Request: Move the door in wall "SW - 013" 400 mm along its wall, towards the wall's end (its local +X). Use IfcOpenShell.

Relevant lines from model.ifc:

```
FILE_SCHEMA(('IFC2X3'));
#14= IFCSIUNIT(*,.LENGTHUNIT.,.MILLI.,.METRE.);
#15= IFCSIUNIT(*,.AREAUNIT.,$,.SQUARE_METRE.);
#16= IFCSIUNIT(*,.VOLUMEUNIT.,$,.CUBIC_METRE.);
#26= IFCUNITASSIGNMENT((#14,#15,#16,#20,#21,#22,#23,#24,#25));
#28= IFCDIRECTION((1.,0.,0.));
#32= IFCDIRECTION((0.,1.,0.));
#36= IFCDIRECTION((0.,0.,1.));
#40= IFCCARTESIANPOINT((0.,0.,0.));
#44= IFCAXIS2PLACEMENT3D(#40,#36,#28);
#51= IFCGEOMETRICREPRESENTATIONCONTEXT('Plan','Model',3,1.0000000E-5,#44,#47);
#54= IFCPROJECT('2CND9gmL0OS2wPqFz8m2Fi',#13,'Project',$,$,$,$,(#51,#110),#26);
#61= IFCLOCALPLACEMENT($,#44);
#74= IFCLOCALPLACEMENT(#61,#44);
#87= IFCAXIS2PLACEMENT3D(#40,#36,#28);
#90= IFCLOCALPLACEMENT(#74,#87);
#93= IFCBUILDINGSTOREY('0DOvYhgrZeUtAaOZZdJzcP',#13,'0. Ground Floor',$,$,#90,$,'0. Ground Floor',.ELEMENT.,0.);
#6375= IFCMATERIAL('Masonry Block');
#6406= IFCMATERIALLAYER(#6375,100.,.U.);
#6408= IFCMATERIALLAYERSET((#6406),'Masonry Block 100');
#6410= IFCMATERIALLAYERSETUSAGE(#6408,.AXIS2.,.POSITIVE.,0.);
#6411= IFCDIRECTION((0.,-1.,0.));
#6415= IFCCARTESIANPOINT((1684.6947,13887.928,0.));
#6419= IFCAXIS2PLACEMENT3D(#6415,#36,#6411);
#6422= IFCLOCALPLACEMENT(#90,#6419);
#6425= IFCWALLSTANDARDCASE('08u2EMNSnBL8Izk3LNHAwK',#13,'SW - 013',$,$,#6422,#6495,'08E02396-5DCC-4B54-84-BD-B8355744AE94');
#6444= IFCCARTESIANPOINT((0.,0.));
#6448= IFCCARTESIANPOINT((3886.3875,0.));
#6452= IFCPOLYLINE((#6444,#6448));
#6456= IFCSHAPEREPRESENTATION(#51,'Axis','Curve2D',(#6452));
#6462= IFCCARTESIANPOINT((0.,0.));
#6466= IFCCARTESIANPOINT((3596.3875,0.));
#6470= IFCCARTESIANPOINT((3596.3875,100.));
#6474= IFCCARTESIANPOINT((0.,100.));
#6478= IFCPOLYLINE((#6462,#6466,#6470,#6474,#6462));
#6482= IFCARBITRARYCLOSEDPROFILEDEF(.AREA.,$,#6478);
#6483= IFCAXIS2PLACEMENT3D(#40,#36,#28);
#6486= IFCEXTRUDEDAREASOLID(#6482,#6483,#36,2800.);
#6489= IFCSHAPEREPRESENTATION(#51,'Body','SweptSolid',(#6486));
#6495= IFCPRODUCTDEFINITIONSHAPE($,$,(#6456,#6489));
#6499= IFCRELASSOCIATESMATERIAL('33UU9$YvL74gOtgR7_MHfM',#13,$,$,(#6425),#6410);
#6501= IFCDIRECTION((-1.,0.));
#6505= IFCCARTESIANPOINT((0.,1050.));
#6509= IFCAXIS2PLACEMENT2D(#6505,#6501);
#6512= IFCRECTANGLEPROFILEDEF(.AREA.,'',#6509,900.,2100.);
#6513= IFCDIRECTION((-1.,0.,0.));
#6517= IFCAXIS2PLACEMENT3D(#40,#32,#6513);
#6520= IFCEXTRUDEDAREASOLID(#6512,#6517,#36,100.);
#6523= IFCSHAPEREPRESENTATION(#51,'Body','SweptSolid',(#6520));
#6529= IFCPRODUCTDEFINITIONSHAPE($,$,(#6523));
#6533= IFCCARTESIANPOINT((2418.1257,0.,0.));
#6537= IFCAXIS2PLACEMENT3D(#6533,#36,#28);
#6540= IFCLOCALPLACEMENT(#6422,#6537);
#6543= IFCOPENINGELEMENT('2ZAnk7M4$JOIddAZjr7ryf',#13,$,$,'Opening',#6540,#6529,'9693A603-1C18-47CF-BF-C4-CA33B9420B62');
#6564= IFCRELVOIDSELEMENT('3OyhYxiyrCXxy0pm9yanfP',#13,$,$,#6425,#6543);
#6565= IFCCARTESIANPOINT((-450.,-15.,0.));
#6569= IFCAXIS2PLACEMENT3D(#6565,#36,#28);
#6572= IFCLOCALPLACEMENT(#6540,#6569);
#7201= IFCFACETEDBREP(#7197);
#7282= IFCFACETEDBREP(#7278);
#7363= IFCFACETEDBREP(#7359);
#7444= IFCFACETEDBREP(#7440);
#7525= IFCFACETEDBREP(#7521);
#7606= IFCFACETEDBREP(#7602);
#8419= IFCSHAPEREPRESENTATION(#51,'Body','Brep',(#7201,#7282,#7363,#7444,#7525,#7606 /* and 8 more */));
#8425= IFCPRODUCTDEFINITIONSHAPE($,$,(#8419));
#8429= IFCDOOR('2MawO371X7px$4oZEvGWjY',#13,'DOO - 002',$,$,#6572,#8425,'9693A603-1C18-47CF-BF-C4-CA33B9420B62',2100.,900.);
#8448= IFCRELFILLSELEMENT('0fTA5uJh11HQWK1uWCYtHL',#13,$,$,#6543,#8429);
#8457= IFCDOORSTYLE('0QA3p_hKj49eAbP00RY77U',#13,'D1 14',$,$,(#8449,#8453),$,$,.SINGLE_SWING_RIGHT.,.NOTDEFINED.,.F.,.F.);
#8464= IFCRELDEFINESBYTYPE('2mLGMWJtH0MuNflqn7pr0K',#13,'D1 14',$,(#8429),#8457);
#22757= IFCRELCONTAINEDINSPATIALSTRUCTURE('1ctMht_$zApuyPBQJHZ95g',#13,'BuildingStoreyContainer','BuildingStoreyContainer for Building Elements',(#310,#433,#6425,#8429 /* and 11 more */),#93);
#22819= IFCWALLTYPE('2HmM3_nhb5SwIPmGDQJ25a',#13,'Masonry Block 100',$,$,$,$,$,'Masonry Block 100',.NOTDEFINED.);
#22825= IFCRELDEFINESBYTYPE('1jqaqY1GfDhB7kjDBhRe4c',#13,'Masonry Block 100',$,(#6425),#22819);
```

```python
import ifcopenshell
import ifcopenshell.api.geometry
import ifcopenshell.util.placement

model = ifcopenshell.open("model.ifc")

door = model.by_guid("2MawO371X7px$4oZEvGWjY")
opening = door.FillsVoids[0].RelatingOpeningElement
wall = opening.VoidsElements[0].RelatingBuildingElement

wall_matrix = ifcopenshell.util.placement.get_local_placement(wall.ObjectPlacement)
shift = wall_matrix[:3, 0] * 400.0
before = ifcopenshell.util.placement.get_local_placement(door.ObjectPlacement)[:3, 3].copy()

# The door is placed relative to its opening, so it follows when the opening moves.
matrix = ifcopenshell.util.placement.get_local_placement(opening.ObjectPlacement)
matrix[:3, 3] += shift
ifcopenshell.api.geometry.edit_object_placement(
    model, product=opening, matrix=matrix, is_si=False, should_transform_children=True
)

after = ifcopenshell.util.placement.get_local_placement(door.ObjectPlacement)[:3, 3]
print("door moved by", (after - before).round(3) + 0.0)

model.write("model_v2.ifc")
```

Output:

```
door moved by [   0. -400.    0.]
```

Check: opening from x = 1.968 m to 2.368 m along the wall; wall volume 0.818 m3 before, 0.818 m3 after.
